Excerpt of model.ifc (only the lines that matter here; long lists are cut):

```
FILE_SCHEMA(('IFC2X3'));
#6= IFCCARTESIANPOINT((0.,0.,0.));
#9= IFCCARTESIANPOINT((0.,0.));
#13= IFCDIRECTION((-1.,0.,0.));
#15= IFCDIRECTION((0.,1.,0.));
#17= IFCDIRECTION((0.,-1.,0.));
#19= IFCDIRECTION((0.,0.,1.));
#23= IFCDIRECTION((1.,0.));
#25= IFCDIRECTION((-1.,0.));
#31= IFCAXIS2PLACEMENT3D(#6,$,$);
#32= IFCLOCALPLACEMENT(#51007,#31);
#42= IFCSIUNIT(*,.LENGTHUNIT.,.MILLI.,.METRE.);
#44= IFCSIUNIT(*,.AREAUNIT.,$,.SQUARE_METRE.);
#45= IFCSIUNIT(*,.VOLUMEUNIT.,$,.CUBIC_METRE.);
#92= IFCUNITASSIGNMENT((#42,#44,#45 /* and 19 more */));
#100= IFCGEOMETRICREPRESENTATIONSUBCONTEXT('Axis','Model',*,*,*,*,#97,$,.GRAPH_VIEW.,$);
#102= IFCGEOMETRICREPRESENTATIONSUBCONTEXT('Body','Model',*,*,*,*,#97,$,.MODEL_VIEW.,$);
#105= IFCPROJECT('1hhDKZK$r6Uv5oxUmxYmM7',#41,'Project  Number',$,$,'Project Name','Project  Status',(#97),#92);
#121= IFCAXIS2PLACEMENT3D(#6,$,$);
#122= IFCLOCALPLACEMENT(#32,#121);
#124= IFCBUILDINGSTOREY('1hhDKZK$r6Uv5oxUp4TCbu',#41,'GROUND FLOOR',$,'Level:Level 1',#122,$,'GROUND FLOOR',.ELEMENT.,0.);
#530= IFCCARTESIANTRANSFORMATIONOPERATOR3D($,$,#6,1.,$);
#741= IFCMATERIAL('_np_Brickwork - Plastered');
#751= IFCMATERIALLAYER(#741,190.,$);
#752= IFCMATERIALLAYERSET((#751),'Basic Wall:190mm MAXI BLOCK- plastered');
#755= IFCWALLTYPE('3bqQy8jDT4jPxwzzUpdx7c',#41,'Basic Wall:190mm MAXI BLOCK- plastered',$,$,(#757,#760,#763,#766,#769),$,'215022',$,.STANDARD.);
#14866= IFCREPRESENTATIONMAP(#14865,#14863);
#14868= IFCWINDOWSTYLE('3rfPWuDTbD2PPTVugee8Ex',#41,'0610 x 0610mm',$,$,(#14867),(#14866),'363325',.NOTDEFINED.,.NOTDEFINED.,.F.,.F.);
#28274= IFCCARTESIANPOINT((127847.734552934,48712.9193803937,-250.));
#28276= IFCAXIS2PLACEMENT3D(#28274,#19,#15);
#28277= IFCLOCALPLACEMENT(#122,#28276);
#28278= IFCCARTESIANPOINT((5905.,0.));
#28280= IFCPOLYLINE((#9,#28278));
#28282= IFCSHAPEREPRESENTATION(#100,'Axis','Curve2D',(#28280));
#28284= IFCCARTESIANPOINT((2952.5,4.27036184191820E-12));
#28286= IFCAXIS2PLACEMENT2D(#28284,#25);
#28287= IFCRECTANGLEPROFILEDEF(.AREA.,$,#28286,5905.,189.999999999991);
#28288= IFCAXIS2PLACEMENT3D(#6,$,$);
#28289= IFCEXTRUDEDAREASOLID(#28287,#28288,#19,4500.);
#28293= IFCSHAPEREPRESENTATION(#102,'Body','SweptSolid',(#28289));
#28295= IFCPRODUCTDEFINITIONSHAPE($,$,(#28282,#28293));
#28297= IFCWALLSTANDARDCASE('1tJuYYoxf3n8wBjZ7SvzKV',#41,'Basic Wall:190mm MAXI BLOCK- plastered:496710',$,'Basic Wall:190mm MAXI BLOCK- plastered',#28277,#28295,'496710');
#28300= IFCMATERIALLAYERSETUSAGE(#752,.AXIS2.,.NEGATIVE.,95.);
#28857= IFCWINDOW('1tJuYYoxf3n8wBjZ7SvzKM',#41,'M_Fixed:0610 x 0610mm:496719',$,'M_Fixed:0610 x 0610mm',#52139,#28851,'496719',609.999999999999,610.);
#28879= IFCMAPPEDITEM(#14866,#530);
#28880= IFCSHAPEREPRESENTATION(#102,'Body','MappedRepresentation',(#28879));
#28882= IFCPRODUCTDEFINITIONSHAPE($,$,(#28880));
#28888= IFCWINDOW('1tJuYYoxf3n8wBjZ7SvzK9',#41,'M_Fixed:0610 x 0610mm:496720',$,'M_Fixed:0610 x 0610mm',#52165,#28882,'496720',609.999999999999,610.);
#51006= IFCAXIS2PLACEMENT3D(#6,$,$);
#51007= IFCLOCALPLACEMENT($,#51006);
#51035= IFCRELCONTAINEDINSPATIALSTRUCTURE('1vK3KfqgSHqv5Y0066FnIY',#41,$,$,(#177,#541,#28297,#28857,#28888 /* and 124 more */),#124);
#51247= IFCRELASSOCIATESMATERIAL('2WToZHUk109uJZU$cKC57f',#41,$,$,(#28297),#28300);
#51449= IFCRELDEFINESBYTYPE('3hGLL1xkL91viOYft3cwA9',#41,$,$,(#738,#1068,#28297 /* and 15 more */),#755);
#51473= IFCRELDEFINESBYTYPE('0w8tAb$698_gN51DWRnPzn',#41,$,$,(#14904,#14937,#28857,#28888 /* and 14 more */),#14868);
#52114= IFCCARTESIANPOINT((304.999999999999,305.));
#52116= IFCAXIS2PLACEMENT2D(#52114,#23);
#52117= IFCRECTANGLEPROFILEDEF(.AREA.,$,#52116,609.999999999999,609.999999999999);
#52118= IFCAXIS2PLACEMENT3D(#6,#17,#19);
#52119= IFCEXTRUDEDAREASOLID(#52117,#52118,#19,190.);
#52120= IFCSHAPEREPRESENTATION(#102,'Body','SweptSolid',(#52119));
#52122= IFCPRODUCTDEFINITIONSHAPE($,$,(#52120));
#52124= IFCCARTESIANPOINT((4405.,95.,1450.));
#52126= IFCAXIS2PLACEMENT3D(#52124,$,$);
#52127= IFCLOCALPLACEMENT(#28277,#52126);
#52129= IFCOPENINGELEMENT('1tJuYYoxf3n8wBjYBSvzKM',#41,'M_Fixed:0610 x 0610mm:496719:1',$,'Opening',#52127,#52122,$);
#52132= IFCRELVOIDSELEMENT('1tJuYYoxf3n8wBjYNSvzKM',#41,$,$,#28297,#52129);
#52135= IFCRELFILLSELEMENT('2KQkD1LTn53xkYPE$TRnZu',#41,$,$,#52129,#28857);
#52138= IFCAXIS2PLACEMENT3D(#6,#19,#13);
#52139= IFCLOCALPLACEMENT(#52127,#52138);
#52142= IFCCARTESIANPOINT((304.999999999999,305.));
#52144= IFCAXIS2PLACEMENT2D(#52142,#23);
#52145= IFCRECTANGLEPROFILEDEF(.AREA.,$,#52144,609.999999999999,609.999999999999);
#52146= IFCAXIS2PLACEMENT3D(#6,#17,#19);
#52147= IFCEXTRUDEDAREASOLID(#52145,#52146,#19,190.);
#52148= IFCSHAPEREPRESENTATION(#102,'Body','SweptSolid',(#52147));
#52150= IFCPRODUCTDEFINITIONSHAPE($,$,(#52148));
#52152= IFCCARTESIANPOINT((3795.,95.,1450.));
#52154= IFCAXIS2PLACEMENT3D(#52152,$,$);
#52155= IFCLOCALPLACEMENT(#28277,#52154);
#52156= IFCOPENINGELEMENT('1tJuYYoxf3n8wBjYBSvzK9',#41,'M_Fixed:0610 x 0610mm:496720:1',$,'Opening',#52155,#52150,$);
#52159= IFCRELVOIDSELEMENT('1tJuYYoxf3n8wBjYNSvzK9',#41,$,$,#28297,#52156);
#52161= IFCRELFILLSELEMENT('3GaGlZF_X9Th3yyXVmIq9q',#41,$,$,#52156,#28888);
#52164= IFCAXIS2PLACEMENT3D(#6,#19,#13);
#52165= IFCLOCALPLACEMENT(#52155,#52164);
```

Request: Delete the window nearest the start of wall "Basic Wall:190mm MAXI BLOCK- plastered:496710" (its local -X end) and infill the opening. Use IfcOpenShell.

```python
import ifcopenshell
import ifcopenshell.api.feature
import ifcopenshell.api.root
import ifcopenshell.geom
import ifcopenshell.util.shape

model = ifcopenshell.open("model.ifc")
settings = ifcopenshell.geom.settings()


def volume(element):
    """Net volume in cubic metres, openings subtracted."""
    shape = ifcopenshell.geom.create_shape(settings, element)
    return ifcopenshell.util.shape.get_volume(shape.geometry)


window = model.by_id(28888)
opening = window.FillsVoids[0].RelatingOpeningElement
wall = opening.VoidsElements[0].RelatingBuildingElement
before = volume(wall)

ifcopenshell.api.root.remove_product(model, product=window)
ifcopenshell.api.feature.remove_feature(model, feature=opening)

after = volume(wall)

print(f"wall volume {before:.3f} -> {after:.3f} m3")

model.write("model_edited.ifc")
```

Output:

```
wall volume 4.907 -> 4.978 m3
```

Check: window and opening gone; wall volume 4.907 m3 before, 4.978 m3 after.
